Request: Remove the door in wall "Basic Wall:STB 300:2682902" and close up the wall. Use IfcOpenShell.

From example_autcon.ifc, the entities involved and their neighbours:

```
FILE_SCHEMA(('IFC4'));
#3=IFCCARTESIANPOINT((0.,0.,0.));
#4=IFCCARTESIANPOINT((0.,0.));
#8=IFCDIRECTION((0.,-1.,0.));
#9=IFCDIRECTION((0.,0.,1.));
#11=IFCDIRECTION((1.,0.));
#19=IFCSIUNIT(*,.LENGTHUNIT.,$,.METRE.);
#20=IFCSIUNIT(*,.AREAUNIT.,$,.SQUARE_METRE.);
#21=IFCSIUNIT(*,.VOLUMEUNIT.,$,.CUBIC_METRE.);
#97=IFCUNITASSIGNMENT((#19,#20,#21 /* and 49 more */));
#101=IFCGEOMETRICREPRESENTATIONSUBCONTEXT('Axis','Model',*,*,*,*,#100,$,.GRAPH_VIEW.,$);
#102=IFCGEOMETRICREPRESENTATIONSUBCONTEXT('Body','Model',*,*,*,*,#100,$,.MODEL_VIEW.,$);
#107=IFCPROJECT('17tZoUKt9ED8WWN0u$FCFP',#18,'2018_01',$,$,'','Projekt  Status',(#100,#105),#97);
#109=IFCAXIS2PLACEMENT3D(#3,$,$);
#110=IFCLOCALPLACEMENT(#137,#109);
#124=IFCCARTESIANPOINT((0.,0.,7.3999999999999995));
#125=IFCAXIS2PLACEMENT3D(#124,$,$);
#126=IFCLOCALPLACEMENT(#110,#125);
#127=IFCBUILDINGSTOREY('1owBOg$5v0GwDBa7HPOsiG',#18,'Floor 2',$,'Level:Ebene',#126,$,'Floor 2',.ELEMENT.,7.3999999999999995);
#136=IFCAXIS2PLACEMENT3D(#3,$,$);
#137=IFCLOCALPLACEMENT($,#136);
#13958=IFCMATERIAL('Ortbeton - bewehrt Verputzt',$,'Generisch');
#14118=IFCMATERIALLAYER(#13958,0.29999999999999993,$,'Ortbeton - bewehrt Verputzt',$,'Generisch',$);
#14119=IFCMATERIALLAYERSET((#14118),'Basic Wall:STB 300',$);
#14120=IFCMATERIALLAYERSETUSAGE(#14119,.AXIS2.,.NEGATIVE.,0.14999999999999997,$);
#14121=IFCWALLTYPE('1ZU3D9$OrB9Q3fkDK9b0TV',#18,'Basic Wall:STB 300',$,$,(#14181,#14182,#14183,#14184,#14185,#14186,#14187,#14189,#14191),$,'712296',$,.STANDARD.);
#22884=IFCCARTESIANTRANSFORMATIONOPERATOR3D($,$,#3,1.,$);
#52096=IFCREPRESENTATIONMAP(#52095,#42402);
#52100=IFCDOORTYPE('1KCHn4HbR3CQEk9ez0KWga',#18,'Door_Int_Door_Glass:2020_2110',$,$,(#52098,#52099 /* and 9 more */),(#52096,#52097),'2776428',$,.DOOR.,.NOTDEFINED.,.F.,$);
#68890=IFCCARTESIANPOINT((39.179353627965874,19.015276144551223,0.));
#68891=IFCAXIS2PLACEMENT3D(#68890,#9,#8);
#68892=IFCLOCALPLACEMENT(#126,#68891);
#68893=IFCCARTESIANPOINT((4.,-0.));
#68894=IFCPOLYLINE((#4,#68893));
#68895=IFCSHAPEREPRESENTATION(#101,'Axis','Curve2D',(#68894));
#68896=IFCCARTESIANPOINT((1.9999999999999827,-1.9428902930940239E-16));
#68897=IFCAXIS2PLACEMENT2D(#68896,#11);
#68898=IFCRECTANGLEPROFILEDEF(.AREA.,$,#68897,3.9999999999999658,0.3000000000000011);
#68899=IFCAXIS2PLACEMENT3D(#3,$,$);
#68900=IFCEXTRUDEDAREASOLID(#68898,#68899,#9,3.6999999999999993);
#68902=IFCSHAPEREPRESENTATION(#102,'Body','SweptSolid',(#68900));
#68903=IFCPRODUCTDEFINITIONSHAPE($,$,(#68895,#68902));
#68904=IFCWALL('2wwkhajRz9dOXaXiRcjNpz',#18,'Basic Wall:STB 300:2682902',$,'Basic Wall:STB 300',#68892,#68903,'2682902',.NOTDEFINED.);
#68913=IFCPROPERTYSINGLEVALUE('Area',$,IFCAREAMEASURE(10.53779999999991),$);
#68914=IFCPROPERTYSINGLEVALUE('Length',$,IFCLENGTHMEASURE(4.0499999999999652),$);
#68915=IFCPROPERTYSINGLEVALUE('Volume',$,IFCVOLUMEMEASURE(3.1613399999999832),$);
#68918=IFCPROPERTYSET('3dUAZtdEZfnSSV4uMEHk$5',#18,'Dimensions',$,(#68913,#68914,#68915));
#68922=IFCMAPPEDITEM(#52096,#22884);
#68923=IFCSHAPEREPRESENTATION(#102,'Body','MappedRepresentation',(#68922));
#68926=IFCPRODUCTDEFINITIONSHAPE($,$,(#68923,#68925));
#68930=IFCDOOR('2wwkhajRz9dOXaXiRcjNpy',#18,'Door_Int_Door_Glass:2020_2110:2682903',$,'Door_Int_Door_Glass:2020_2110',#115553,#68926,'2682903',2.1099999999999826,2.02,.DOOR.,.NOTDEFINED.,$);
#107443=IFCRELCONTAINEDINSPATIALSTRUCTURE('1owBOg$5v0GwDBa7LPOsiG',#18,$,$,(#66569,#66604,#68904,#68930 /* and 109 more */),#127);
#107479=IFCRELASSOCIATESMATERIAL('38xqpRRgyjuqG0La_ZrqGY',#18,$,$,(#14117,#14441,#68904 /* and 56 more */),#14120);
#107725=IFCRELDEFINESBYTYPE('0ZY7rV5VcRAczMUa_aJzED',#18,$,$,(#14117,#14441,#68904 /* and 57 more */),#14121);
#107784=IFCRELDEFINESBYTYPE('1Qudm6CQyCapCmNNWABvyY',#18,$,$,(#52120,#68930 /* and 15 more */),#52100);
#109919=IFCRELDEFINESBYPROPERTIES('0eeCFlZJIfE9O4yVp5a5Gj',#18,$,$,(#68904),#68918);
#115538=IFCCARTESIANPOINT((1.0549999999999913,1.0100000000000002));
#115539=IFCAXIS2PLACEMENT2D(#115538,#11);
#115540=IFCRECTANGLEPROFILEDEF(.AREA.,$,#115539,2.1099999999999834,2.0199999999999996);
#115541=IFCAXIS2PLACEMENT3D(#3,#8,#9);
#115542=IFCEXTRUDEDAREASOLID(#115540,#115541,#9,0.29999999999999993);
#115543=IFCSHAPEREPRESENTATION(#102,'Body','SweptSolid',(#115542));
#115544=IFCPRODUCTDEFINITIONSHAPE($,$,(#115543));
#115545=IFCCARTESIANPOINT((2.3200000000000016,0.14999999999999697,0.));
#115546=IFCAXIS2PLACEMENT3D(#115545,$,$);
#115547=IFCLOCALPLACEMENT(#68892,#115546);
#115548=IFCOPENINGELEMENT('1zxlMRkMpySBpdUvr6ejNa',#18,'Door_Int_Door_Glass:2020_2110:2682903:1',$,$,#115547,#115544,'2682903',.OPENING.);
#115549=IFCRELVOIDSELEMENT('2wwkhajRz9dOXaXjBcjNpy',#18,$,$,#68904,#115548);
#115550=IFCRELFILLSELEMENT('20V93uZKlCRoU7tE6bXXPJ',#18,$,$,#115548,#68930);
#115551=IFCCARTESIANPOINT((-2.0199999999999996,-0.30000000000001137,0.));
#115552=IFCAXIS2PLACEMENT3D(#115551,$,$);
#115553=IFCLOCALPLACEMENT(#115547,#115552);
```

```python
import ifcopenshell
import ifcopenshell.api.feature
import ifcopenshell.api.pset
import ifcopenshell.api.root
import ifcopenshell.geom
import ifcopenshell.util.element
import ifcopenshell.util.shape
import ifcopenshell.util.unit

model = ifcopenshell.open("example_autcon.ifc")
area_scale = ifcopenshell.util.unit.calculate_unit_scale(model, "AREAUNIT")
volume_scale = ifcopenshell.util.unit.calculate_unit_scale(model, "VOLUMEUNIT")
settings = ifcopenshell.geom.settings()


def volume(element):
    """Net volume in cubic metres, openings subtracted."""
    shape = ifcopenshell.geom.create_shape(settings, element)
    return ifcopenshell.util.shape.get_volume(shape.geometry)


door = model.by_guid("2wwkhajRz9dOXaXiRcjNpy")
opening = door.FillsVoids[0].RelatingOpeningElement
wall = opening.VoidsElements[0].RelatingBuildingElement
before = volume(wall)

ifcopenshell.api.root.remove_product(model, product=door)
ifcopenshell.api.feature.remove_feature(model, feature=opening)

after = volume(wall)
thickness = 0.3  # wall thickness in metres

# Update the wall's stored quantities.
pset = model.by_id(ifcopenshell.util.element.get_pset(wall, "Dimensions", should_inherit=False)["id"])
ifcopenshell.api.pset.edit_pset(model, pset=pset, properties={
    "Area": model.create_entity("IfcAreaMeasure", after / thickness / area_scale),
    "Volume": model.create_entity("IfcVolumeMeasure", after / volume_scale),
})

print(f"wall volume {before:.3f} -> {after:.3f} m3")

model.write("example_autcon-out.ifc")
```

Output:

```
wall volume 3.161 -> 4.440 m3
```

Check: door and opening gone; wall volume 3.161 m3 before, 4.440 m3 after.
